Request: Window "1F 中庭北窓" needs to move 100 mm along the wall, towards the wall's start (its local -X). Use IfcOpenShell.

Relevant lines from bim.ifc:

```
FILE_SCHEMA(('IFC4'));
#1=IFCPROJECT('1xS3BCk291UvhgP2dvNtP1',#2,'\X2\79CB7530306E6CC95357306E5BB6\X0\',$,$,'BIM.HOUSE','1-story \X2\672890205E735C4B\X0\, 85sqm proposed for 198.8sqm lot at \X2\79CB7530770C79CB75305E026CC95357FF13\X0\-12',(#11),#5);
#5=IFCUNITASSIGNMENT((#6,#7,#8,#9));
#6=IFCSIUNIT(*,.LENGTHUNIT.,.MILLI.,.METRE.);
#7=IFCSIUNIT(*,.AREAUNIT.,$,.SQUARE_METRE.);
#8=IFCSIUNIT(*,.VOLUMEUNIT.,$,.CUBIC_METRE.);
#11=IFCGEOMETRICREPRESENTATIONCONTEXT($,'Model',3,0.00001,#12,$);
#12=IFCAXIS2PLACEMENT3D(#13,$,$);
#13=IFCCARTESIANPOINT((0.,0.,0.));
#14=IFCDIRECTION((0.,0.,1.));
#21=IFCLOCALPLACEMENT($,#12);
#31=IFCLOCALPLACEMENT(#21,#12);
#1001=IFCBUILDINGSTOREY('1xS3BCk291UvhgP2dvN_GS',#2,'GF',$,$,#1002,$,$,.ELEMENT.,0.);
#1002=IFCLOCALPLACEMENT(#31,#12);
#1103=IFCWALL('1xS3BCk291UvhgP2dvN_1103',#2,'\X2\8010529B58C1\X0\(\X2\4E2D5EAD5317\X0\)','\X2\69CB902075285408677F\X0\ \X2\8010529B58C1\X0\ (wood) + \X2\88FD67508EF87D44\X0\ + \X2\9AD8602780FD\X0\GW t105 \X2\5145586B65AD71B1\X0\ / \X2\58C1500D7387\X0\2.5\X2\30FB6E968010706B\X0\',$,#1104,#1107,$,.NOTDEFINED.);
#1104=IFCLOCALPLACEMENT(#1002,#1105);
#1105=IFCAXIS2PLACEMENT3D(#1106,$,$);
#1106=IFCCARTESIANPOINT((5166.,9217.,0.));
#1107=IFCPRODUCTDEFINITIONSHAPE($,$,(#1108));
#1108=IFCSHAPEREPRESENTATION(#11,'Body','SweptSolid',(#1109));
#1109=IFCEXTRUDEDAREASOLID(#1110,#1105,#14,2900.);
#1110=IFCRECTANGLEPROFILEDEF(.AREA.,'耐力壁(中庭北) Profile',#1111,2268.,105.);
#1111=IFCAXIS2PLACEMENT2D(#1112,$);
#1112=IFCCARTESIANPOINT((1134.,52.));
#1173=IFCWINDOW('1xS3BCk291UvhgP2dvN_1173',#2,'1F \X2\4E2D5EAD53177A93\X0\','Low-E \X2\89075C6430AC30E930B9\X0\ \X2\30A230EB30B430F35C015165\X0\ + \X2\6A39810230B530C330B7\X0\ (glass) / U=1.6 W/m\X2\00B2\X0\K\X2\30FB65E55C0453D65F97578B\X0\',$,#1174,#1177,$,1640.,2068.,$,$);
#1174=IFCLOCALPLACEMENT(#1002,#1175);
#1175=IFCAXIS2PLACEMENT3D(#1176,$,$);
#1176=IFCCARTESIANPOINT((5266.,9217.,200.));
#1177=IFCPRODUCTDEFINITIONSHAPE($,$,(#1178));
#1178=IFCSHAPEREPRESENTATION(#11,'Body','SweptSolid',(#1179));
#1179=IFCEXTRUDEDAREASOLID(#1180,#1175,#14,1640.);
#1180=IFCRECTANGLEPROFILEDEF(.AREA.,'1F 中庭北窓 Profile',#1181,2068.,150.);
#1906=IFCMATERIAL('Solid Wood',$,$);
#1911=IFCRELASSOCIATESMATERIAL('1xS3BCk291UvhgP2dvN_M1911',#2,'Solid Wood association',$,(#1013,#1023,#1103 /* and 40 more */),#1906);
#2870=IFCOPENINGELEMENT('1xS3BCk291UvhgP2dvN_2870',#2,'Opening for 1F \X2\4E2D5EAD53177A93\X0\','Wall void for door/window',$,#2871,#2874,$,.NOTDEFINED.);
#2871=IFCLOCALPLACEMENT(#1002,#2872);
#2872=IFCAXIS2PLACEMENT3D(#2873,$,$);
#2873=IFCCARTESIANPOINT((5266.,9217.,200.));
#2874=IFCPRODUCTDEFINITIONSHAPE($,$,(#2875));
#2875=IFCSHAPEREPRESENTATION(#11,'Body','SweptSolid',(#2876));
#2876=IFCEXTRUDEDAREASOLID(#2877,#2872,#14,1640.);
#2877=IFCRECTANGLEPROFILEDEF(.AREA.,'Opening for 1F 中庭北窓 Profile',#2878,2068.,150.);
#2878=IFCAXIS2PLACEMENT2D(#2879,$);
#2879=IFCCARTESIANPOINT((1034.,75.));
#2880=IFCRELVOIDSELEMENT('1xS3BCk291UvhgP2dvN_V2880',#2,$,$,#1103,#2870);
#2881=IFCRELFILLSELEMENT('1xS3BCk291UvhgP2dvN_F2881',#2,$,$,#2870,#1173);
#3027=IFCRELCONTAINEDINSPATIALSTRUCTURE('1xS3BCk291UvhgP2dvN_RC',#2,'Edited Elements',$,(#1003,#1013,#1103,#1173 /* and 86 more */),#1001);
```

```python
import ifcopenshell
import ifcopenshell.api.geometry
import ifcopenshell.util.placement

model = ifcopenshell.open("bim.ifc")

window = model.by_guid("1xS3BCk291UvhgP2dvN_1173")
opening = window.FillsVoids[0].RelatingOpeningElement
wall = opening.VoidsElements[0].RelatingBuildingElement

wall_matrix = ifcopenshell.util.placement.get_local_placement(wall.ObjectPlacement)
shift = wall_matrix[:3, 0] * -100.0
before = ifcopenshell.util.placement.get_local_placement(window.ObjectPlacement)[:3, 3].copy()

# The window is not placed relative to its opening, so move both.
for product in (opening, window):
    matrix = ifcopenshell.util.placement.get_local_placement(product.ObjectPlacement)
    matrix[:3, 3] += shift
    ifcopenshell.api.geometry.edit_object_placement(model, product=product, matrix=matrix, is_si=False)

after = ifcopenshell.util.placement.get_local_placement(window.ObjectPlacement)[:3, 3]
print("window moved by", (after - before).round(3) + 0.0)

model.write("bim_v2.ifc")
```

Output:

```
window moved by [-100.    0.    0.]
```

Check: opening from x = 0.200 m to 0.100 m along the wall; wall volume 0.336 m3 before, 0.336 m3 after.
